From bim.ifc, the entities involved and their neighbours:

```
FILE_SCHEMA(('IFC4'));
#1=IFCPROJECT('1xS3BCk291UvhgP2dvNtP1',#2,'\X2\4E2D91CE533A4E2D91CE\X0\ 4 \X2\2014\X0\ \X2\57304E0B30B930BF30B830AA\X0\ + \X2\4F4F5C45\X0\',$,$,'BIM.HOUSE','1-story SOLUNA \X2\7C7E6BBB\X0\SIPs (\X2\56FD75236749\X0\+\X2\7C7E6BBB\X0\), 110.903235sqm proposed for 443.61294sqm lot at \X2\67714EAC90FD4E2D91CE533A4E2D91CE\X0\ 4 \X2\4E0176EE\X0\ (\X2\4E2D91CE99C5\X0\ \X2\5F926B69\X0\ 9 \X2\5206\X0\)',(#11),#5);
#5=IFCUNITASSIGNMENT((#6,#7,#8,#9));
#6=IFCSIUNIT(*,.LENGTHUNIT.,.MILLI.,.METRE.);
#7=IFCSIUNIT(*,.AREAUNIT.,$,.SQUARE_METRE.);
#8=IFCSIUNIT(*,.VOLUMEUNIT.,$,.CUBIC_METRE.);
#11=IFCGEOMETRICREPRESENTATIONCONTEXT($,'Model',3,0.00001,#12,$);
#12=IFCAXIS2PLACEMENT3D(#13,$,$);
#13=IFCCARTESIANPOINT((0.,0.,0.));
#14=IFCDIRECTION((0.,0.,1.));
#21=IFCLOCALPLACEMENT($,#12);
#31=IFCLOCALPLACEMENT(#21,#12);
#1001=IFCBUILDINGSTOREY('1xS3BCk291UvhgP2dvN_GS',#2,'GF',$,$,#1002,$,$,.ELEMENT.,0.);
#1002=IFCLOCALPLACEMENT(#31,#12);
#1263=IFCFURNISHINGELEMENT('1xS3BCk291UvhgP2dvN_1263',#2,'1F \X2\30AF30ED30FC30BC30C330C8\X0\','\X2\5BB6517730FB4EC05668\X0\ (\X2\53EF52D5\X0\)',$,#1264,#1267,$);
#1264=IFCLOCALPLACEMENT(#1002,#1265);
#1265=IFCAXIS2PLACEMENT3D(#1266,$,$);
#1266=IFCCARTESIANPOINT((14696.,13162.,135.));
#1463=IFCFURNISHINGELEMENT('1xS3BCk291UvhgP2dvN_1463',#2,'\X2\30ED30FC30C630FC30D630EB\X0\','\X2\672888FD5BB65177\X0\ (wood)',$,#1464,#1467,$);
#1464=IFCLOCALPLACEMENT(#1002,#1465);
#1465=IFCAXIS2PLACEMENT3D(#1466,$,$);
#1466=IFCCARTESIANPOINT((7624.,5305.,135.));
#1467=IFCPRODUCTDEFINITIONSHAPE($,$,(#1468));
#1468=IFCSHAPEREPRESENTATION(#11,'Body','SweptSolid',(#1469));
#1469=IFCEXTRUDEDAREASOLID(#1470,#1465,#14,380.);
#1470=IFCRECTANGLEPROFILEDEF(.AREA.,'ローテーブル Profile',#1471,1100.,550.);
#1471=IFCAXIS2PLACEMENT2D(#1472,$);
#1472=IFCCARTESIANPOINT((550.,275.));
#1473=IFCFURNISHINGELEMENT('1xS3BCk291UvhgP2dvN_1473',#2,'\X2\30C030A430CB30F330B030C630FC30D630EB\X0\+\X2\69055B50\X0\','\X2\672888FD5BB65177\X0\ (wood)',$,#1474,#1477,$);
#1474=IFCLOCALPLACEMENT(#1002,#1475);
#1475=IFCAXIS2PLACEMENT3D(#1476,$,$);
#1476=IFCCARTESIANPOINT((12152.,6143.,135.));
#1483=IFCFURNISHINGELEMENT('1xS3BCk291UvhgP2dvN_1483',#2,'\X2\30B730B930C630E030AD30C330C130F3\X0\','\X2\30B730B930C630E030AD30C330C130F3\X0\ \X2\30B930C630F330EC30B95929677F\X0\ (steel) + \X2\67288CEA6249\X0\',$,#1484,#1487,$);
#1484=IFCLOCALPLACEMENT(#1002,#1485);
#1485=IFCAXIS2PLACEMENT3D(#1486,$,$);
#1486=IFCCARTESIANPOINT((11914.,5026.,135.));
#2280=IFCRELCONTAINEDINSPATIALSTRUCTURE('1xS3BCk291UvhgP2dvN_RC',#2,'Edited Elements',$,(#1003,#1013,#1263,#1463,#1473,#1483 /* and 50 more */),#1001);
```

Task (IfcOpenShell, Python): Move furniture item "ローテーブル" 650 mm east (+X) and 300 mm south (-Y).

```python
import ifcopenshell
import ifcopenshell.api.geometry
import ifcopenshell.util.placement

model = ifcopenshell.open("bim.ifc")

item = model.by_guid("1xS3BCk291UvhgP2dvN_1463")
matrix = ifcopenshell.util.placement.get_local_placement(item.ObjectPlacement)
matrix[0, 3] += 650.0
matrix[1, 3] -= 300.0
ifcopenshell.api.geometry.edit_object_placement(model, product=item, matrix=matrix, is_si=False)

print(ifcopenshell.util.placement.get_local_placement(item.ObjectPlacement).round(3) + 0.0)

model.write("bim_updated.ifc")
```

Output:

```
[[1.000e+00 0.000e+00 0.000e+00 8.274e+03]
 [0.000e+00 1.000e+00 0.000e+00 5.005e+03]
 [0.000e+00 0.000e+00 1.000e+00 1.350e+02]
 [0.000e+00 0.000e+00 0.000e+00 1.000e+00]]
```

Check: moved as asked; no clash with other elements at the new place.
